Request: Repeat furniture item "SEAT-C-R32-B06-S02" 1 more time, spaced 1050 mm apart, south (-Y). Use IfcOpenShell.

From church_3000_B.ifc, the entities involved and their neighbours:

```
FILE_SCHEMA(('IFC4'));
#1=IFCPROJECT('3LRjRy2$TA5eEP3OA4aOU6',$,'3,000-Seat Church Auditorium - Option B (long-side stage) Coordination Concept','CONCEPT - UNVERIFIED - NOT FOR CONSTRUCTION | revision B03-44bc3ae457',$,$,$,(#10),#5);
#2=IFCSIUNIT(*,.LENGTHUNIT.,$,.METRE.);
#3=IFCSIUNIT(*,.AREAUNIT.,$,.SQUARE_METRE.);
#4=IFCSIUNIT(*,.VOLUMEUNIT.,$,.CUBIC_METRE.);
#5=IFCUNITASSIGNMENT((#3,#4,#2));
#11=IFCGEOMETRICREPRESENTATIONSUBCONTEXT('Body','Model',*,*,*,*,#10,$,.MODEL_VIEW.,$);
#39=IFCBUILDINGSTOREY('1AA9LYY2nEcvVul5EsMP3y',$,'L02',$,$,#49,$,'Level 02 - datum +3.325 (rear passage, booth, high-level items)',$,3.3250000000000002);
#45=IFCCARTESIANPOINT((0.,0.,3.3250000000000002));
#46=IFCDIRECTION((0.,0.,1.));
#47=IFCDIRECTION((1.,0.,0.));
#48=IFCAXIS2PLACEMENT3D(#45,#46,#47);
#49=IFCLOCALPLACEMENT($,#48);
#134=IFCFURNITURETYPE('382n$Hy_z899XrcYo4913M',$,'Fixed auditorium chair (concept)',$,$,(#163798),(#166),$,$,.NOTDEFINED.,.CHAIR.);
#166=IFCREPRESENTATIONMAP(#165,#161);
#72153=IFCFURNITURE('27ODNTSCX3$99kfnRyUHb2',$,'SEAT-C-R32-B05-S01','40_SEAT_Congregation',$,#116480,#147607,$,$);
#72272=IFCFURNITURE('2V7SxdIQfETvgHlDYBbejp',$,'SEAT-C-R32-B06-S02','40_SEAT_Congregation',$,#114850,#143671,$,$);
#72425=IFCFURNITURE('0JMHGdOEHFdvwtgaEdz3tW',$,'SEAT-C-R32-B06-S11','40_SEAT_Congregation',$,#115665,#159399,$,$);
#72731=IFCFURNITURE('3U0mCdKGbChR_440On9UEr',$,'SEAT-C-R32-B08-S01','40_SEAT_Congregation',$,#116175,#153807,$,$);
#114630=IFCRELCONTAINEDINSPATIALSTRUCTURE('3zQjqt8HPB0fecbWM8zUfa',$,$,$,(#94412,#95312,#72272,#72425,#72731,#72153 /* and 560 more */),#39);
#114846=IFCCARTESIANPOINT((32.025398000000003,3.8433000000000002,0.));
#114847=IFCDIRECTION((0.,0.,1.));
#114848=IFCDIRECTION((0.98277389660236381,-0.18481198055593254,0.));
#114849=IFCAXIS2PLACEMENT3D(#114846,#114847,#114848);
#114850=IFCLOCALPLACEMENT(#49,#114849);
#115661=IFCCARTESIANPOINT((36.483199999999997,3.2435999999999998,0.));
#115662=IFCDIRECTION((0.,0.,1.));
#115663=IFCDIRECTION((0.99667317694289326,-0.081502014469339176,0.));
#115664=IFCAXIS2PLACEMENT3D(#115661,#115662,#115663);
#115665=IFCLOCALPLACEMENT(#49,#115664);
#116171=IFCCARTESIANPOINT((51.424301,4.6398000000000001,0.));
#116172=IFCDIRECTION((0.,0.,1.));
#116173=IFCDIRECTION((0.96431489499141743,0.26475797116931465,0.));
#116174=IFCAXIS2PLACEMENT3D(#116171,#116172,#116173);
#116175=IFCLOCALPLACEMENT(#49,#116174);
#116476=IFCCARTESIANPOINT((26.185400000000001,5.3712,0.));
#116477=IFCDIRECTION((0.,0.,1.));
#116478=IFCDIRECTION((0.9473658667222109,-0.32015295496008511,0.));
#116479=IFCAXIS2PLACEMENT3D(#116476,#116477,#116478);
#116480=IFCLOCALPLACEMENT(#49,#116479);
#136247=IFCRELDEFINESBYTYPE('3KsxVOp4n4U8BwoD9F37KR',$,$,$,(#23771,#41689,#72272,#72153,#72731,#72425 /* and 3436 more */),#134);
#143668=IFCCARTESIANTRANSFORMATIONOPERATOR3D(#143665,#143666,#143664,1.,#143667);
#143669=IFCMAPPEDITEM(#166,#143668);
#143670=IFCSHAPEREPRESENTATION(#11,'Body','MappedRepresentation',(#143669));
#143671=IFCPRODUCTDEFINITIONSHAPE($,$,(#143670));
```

```python
import numpy as np
import ifcopenshell
import ifcopenshell.api.geometry
import ifcopenshell.api.root
import ifcopenshell.util.element
import ifcopenshell.util.placement
import ifcopenshell.util.unit

model = ifcopenshell.open("church_3000_B.ifc")
unit_scale = ifcopenshell.util.unit.calculate_unit_scale(model)

source = model.by_id(72272)
base = ifcopenshell.util.placement.get_local_placement(source.ObjectPlacement)
step = np.array([0.0, -1.0, 0.0]) * 1.05 / unit_scale

for i in range(1, 2):
    copy = ifcopenshell.api.root.copy_class(model, product=source)
    copy.Representation = ifcopenshell.util.element.copy_deep(
        model, source.Representation, exclude=["IfcGeometricRepresentationContext", "IfcRepresentationMap"]
    )
    matrix = base.copy()
    matrix[:3, 3] += i * step
    print("added at", matrix[:3, 3].round(3) + 0.0)
    ifcopenshell.api.geometry.edit_object_placement(model, product=copy, matrix=matrix, is_si=False)

model.write("church_3000_B_rev.ifc")
```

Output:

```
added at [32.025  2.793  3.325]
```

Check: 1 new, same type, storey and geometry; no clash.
